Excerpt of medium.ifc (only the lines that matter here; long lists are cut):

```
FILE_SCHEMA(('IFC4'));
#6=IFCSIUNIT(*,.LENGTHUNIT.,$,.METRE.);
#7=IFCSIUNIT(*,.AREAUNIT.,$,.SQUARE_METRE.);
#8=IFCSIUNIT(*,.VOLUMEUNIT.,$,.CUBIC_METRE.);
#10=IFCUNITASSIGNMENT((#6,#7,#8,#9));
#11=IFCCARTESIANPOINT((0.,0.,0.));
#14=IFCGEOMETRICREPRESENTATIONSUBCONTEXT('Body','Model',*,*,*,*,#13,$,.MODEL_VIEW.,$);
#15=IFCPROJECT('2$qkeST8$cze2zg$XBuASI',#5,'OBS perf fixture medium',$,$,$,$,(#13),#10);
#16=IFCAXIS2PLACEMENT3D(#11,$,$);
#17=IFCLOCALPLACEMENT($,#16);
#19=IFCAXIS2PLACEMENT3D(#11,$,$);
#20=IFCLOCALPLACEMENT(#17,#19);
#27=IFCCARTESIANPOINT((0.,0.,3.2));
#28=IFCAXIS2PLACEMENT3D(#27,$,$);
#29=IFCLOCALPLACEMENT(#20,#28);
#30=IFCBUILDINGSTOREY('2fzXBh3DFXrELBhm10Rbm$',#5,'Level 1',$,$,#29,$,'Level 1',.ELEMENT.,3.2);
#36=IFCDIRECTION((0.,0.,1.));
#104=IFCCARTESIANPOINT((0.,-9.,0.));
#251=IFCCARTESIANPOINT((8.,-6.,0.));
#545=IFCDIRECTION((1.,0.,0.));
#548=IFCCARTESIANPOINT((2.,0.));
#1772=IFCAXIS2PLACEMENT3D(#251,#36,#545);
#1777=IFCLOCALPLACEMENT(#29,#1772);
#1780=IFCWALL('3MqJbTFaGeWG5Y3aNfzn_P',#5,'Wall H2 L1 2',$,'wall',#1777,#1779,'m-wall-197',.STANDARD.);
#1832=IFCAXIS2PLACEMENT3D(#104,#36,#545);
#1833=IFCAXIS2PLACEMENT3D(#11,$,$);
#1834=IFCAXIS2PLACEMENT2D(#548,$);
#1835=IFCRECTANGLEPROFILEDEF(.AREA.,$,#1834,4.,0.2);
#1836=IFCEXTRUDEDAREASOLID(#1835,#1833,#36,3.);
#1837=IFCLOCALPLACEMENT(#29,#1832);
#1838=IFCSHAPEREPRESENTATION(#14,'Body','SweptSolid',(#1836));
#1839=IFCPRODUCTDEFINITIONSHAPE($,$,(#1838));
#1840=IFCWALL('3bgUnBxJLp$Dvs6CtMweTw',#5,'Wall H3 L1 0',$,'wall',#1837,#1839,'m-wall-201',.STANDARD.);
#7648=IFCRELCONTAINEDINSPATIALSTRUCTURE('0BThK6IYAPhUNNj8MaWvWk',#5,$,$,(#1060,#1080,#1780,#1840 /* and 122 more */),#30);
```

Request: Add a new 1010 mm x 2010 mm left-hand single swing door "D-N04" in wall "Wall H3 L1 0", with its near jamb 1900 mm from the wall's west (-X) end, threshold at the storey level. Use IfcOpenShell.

```python
import numpy as np
import ifcopenshell
import ifcopenshell.api.feature
import ifcopenshell.api.geometry
import ifcopenshell.api.root
import ifcopenshell.api.spatial
import ifcopenshell.geom
import ifcopenshell.util.element
import ifcopenshell.util.placement
import ifcopenshell.util.representation
import ifcopenshell.util.shape
import ifcopenshell.util.unit

model = ifcopenshell.open("medium.ifc")
unit_scale = ifcopenshell.util.unit.calculate_unit_scale(model)
settings = ifcopenshell.geom.settings()


def volume(element):
    """Net volume in cubic metres, openings subtracted."""
    shape = ifcopenshell.geom.create_shape(settings, element)
    return ifcopenshell.util.shape.get_volume(shape.geometry)


wall = model.by_guid("3bgUnBxJLp$Dvs6CtMweTw")
storey = ifcopenshell.util.element.get_container(wall, ifc_class="IfcBuildingStorey")
context = ifcopenshell.util.representation.get_context(model, "Model", "Body", "MODEL_VIEW")
before = volume(wall)

width, height, from_end, sill = 1.01, 2.01, 1.9, 0.0  # metres

# The wall runs along its own X axis, and the end named is its -X end.
wall_shape = ifcopenshell.geom.create_shape(settings, wall)
x, y, z = ifcopenshell.util.shape.get_vertices(wall_shape.geometry).T
start = x.min() + from_end
face, thickness = float(y.min()), float(y.max() - y.min())
wall_matrix = ifcopenshell.util.placement.get_local_placement(wall.ObjectPlacement)
level = ifcopenshell.util.placement.get_local_placement(storey.ObjectPlacement)[2, 3]


def in_wall(x, y):
    """Placement at x, y metres in the wall's axes, at sill height."""
    matrix = wall_matrix.copy()
    matrix[:, 3] = wall_matrix @ np.array([x / unit_scale, y / unit_scale, 0.0, 1.0])
    matrix[2, 3] = level + sill / unit_scale
    return matrix


# Opening: a box that overshoots both wall faces by 50 mm.
opening = ifcopenshell.api.root.create_entity(model, ifc_class="IfcOpeningElement", predefined_type="OPENING")
box = ifcopenshell.api.geometry.add_wall_representation(
    model, context=context, length=width, height=height, thickness=thickness + 0.1
)
ifcopenshell.api.geometry.assign_representation(model, product=opening, representation=box)
ifcopenshell.api.geometry.edit_object_placement(model, product=opening, matrix=in_wall(start, face - 0.05), is_si=False)
ifcopenshell.api.feature.add_feature(model, feature=opening, element=wall)

door = ifcopenshell.api.root.create_entity(model, ifc_class="IfcDoor", name="D-N04", predefined_type="DOOR")
door.OverallWidth, door.OverallHeight = width / unit_scale, height / unit_scale
door.OperationType = "SINGLE_SWING_LEFT"
body = ifcopenshell.api.geometry.add_door_representation(
    model,
    context=context,
    overall_width=door.OverallWidth,
    overall_height=door.OverallHeight,
    operation_type="SINGLE_SWING_LEFT",
    lining_properties={"LiningDepth": thickness / unit_scale, "ThresholdDepth": thickness / unit_scale},
)
ifcopenshell.api.geometry.assign_representation(model, product=door, representation=body)
ifcopenshell.api.spatial.assign_container(model, products=[door], relating_structure=storey)
ifcopenshell.api.feature.add_filling(model, opening=opening, element=door)

# The lining spans the wall, so the door starts at the wall face.
ifcopenshell.api.geometry.edit_object_placement(model, product=door, matrix=in_wall(start, face), is_si=False)

after = volume(wall)

print(f"wall volume {before:.3f} -> {after:.3f} m3")

model.write("medium_v2.ifc")
```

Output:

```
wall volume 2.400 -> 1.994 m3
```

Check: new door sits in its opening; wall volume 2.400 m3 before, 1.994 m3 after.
